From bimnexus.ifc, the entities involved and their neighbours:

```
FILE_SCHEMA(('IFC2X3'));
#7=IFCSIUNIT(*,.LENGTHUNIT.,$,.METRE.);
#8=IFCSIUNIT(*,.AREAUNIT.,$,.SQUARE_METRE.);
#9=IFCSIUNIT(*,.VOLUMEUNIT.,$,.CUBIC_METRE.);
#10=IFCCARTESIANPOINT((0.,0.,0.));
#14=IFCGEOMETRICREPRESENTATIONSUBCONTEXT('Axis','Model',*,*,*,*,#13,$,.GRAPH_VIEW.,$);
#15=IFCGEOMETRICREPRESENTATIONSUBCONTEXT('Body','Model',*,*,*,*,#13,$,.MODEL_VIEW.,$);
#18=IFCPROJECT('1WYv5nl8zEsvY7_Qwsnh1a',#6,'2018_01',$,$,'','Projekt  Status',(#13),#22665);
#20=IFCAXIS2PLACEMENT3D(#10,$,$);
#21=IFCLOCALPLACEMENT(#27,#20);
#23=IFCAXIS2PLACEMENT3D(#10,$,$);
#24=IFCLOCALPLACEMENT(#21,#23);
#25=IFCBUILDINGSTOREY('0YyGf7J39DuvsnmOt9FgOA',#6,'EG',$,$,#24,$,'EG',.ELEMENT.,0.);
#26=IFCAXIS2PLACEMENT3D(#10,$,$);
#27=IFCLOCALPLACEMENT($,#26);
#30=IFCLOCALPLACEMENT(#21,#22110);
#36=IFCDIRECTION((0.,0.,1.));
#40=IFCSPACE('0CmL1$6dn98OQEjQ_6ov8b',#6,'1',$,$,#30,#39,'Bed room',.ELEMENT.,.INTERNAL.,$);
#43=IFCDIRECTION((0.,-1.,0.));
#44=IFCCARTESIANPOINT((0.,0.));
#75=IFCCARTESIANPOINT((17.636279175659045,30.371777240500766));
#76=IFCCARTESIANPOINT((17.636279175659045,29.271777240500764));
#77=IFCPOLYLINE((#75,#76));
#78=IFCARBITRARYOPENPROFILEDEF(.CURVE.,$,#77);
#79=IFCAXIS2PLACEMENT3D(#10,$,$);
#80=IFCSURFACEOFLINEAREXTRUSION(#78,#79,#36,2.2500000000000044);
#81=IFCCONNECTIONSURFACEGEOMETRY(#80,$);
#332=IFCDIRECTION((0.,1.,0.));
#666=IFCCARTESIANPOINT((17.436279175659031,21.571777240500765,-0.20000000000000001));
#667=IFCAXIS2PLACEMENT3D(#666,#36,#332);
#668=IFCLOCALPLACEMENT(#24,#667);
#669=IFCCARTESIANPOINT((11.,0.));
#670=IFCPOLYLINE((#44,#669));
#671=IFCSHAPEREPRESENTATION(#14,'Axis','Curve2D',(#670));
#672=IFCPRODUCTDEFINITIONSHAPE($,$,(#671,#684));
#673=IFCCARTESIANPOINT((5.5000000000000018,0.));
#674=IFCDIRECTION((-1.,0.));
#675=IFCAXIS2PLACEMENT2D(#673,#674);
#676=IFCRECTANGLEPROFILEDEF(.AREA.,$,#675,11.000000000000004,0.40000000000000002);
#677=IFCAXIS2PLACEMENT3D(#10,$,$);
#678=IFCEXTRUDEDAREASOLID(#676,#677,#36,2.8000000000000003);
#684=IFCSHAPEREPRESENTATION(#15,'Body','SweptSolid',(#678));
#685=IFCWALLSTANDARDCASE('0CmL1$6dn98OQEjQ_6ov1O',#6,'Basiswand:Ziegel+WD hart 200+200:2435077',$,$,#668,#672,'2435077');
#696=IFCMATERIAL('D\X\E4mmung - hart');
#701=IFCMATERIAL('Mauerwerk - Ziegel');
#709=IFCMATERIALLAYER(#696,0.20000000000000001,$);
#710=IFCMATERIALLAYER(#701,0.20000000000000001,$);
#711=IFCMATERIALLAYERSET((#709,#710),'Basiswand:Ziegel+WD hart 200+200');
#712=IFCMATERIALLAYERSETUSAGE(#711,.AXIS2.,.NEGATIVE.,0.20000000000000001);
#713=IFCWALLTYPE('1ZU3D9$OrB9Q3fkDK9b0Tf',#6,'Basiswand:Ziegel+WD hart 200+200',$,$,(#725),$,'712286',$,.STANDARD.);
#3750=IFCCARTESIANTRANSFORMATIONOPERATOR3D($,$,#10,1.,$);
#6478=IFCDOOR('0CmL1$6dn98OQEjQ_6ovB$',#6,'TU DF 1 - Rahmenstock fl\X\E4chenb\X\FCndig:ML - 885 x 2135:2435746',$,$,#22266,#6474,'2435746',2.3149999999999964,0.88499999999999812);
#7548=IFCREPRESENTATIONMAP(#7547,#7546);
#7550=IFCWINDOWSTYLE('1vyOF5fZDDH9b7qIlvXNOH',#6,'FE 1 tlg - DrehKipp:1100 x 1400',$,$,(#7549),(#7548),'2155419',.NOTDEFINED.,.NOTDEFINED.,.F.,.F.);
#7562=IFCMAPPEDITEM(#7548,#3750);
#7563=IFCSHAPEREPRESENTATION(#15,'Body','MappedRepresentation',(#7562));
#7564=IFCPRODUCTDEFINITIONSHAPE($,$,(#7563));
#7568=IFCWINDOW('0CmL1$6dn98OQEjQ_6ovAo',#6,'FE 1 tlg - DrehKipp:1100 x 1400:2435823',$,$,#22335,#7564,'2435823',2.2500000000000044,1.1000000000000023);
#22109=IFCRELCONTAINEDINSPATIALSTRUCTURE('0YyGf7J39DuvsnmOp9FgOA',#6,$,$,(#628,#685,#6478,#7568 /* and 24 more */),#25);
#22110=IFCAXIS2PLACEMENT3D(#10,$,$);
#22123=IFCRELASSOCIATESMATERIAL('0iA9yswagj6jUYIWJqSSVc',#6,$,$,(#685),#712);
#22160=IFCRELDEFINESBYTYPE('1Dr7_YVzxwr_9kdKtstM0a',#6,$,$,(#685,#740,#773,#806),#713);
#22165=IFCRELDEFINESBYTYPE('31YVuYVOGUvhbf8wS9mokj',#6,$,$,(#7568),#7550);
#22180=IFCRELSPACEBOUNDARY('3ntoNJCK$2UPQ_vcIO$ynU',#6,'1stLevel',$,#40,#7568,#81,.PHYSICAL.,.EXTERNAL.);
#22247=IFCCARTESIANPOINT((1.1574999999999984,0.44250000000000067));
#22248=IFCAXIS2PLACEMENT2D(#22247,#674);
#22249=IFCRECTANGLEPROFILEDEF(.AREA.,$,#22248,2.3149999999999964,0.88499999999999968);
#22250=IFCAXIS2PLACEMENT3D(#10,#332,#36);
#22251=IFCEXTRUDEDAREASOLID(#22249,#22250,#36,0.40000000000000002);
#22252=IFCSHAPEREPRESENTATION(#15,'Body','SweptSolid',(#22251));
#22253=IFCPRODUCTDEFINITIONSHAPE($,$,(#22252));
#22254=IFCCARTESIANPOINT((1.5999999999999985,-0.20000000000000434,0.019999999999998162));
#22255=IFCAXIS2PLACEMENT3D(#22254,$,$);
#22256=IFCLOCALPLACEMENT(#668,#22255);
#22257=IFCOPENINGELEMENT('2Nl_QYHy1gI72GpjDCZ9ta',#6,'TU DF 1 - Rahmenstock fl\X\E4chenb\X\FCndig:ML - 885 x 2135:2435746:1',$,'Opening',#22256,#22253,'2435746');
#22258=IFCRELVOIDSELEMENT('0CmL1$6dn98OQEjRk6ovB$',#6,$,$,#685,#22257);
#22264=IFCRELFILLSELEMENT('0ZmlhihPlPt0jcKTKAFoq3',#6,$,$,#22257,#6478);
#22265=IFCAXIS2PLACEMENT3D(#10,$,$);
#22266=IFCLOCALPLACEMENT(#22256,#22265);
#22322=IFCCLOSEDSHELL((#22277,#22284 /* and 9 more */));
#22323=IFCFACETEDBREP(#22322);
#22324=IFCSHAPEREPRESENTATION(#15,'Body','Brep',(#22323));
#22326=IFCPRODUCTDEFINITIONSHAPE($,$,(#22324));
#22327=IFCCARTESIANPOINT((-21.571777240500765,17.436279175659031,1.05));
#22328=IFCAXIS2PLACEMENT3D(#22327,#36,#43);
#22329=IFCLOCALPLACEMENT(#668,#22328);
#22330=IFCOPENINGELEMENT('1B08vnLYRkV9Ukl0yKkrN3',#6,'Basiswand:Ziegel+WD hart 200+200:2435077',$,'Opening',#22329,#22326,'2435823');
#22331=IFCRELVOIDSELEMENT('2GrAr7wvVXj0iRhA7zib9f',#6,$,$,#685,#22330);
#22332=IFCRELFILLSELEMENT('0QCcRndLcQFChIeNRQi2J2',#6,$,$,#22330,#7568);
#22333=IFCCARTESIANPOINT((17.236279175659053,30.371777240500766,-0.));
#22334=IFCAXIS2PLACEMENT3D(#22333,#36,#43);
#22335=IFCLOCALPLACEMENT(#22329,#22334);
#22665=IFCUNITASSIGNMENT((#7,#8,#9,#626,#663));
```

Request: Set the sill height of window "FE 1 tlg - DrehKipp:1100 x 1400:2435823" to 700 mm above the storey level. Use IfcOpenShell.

```python
import numpy as np
import ifcopenshell
import ifcopenshell.api.geometry
import ifcopenshell.geom
import ifcopenshell.util.element
import ifcopenshell.util.placement
import ifcopenshell.util.shape
import ifcopenshell.util.unit

model = ifcopenshell.open("bimnexus.ifc")
unit_scale = ifcopenshell.util.unit.calculate_unit_scale(model)

window = model.by_guid("0CmL1$6dn98OQEjQ_6ovAo")
opening = window.FillsVoids[0].RelatingOpeningElement
storey = ifcopenshell.util.element.get_container(window, ifc_class="IfcBuildingStorey")
level = ifcopenshell.util.placement.get_local_placement(storey.ObjectPlacement)[2, 3]

# The opening's origin need not be at the sill, so measure its lowest point.
shape = ifcopenshell.geom.create_shape(ifcopenshell.geom.settings(), opening)
bottom = ifcopenshell.util.shape.get_shape_bottom_elevation(shape, shape.geometry) / unit_scale
dz = level + 0.7 / unit_scale - bottom

shift = np.array([0.0, 0.0, dz])
# The window is placed relative to its opening, so it follows when the opening moves.
matrix = ifcopenshell.util.placement.get_local_placement(opening.ObjectPlacement)
matrix[:3, 3] += shift
ifcopenshell.api.geometry.edit_object_placement(
    model, product=opening, matrix=matrix, is_si=False, should_transform_children=True
)

# Space boundary surfaces are stored in each space's coordinates; move them too.
for rel in window.ProvidesBoundaries:
    if not rel.ConnectionGeometry:
        continue
    surface = rel.ConnectionGeometry.SurfaceOnRelatingElement
    space_matrix = ifcopenshell.util.placement.get_local_placement(rel.RelatingSpace.ObjectPlacement)
    point = np.array(surface.Position.Location.Coordinates) + space_matrix[:3, :3].T @ shift
    surface.Position = model.createIfcAxis2Placement3D(
        model.createIfcCartesianPoint(point.tolist()), surface.Position.Axis, surface.Position.RefDirection
    )

print(f"moved by {dz * unit_scale:+.3f} m")

model.write("bimnexus_edited.ifc")
```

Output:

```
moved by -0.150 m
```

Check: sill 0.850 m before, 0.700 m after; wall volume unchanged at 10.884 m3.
